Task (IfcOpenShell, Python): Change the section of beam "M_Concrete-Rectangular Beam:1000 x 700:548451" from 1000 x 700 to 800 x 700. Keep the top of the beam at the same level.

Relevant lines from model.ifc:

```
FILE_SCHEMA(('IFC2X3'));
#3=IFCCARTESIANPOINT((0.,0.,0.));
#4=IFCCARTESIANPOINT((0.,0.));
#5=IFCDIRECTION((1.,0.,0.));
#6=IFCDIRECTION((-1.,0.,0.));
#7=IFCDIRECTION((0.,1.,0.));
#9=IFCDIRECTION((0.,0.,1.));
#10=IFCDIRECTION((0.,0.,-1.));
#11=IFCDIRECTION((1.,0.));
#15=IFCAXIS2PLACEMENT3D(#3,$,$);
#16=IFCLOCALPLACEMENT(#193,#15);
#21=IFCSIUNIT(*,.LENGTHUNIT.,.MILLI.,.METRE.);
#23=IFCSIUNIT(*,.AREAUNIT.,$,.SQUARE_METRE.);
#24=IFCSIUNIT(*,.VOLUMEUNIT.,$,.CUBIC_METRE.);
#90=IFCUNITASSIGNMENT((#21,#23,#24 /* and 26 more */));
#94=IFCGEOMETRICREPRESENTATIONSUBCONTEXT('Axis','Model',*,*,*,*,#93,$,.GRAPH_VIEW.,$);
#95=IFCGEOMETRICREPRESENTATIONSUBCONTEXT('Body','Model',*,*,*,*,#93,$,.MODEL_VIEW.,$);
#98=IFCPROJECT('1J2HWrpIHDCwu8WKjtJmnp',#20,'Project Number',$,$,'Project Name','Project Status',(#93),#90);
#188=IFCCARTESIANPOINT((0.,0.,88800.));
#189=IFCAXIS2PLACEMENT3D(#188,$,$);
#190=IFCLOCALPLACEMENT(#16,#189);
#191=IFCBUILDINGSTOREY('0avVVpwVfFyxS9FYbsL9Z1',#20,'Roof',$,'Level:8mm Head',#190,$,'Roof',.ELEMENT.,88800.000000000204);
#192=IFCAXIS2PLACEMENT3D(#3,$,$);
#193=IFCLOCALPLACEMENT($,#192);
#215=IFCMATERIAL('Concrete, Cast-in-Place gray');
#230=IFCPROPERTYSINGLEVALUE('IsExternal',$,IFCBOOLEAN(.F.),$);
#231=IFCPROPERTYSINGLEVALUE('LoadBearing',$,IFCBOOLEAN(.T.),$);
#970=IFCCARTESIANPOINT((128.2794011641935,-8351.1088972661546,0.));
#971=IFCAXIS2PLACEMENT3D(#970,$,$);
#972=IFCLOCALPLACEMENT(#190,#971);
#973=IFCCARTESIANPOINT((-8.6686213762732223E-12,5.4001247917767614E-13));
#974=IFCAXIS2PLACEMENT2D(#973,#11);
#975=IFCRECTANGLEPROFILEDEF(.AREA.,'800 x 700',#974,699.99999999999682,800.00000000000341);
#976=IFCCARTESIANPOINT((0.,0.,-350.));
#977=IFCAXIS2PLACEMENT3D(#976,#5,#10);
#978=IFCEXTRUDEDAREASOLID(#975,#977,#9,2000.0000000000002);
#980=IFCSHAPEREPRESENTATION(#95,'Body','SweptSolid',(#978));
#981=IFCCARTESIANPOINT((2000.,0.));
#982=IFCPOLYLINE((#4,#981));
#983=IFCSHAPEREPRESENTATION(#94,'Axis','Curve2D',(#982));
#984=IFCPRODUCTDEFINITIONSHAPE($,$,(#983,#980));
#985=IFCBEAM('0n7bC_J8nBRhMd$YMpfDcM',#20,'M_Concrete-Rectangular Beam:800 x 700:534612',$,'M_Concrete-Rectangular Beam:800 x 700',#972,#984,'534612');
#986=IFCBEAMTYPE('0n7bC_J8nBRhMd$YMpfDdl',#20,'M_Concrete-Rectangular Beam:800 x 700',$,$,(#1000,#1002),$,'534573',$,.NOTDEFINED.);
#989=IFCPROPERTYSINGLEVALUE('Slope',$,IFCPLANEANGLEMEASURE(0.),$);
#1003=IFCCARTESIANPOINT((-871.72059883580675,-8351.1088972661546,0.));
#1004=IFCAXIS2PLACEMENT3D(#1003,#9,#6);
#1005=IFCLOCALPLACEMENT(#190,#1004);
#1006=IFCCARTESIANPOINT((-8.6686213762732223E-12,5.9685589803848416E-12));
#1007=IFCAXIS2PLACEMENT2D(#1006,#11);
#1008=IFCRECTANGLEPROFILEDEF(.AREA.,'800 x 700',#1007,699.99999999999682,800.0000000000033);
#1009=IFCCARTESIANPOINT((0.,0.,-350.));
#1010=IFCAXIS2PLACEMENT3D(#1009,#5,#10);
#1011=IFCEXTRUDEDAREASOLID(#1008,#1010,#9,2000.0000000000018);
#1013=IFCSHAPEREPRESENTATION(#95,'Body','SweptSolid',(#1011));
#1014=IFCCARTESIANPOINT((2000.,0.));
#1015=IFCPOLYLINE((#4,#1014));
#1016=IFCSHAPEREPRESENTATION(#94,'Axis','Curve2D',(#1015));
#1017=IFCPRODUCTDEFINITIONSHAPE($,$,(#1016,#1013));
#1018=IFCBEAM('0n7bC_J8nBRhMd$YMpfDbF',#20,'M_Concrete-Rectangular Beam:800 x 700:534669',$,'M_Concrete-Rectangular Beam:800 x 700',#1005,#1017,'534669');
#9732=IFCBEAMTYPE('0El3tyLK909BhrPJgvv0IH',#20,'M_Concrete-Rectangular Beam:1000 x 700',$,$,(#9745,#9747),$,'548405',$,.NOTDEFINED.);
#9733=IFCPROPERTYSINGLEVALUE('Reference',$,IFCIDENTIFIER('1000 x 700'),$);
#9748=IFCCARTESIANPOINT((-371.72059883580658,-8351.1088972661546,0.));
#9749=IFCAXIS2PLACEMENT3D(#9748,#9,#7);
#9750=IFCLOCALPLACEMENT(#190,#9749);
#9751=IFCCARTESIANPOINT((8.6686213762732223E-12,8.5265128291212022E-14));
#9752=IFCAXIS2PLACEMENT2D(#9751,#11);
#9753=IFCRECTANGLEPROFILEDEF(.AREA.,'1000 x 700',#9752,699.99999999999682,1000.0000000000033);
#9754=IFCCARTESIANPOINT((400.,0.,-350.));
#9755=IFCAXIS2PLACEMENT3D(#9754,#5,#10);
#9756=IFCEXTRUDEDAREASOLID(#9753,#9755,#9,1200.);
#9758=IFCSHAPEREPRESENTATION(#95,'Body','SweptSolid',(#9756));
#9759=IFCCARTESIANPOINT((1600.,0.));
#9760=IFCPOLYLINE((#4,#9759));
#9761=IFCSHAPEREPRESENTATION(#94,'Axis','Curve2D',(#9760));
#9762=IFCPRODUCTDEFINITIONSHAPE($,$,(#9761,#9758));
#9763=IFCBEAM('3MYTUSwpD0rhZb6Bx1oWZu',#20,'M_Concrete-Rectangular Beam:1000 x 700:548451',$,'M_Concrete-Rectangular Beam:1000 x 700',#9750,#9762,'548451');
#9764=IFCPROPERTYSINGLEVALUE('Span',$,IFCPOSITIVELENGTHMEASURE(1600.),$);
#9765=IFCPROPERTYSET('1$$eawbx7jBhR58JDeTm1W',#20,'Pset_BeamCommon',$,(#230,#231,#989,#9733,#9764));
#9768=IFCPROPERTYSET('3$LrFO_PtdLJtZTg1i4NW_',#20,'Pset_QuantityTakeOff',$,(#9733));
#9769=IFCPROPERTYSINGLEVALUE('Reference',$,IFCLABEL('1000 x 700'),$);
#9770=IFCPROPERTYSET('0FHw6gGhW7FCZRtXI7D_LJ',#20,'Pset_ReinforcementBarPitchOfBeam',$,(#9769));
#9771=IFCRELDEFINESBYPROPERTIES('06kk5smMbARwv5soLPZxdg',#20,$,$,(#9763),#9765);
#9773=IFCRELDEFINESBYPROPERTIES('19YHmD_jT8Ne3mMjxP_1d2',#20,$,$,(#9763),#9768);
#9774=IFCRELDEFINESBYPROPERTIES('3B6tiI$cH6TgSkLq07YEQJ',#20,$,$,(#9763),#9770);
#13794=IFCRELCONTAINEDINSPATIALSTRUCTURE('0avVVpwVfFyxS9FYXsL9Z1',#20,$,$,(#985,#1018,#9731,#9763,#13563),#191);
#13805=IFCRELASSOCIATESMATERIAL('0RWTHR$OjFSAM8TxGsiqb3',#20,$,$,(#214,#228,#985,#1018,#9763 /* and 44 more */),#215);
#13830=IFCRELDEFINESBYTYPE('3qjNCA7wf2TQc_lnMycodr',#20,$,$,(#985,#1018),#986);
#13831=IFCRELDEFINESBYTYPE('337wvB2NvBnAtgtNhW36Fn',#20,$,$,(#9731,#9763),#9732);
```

```python
import ifcopenshell
import ifcopenshell.api.pset
import ifcopenshell.api.type
import ifcopenshell.util.element
import ifcopenshell.util.representation

model = ifcopenshell.open("model.ifc")

member = model.by_guid("3MYTUSwpD0rhZb6Bx1oWZu")
source = next(p for p in model.by_type("IfcRectangleProfileDef") if p.ProfileName == "800 x 700")

body = ifcopenshell.util.representation.get_representation(member, "Model", "Body")
solid = body.Items[0]
old_profile = solid.SweptArea

# Copy the section's sizes but keep this member's own profile position.
profile = ifcopenshell.util.element.copy(model, source)
# Profiles are centred, so shift by half the change in depth to hold the top.
shift = (old_profile.XDim - profile.XDim) / 2
x, y = old_profile.Position.Location.Coordinates
up = (-1.0, 0.0)  # upwards, in the solid's own plane
location = model.createIfcCartesianPoint((x + up[0] * shift, y + up[1] * shift))
profile.Position = model.createIfcAxis2Placement2D(location, old_profile.Position.RefDirection)
solid.SweptArea = profile
if not model.get_total_inverses(old_profile):
    ifcopenshell.util.element.remove_deep2(model, old_profile)

new_type = model.by_guid("0n7bC_J8nBRhMd$YMpfDdl")
ifcopenshell.api.type.assign_type(
    model, related_objects=[member], relating_type=new_type, should_map_representations=False
)
member.Name = member.Name.replace("1000 x 700", "800 x 700")
member.ObjectType = "M_Concrete-Rectangular Beam:800 x 700"
pset = model.by_id(ifcopenshell.util.element.get_pset(member, "Pset_BeamCommon", should_inherit=False)["id"])
ifcopenshell.api.pset.edit_pset(model, pset=pset, properties={"Reference": "800 x 700"})
pset = model.by_id(ifcopenshell.util.element.get_pset(member, "Pset_QuantityTakeOff", should_inherit=False)["id"])
ifcopenshell.api.pset.edit_pset(model, pset=pset, properties={"Reference": "800 x 700"})
pset = model.by_id(ifcopenshell.util.element.get_pset(member, "Pset_ReinforcementBarPitchOfBeam", should_inherit=False)["id"])
ifcopenshell.api.pset.edit_pset(model, pset=pset, properties={"Reference": "800 x 700"})

print(solid.SweptArea)

model.write("model_rev.ifc")
```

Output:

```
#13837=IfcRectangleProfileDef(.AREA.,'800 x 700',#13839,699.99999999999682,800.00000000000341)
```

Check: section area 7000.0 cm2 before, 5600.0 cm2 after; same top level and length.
